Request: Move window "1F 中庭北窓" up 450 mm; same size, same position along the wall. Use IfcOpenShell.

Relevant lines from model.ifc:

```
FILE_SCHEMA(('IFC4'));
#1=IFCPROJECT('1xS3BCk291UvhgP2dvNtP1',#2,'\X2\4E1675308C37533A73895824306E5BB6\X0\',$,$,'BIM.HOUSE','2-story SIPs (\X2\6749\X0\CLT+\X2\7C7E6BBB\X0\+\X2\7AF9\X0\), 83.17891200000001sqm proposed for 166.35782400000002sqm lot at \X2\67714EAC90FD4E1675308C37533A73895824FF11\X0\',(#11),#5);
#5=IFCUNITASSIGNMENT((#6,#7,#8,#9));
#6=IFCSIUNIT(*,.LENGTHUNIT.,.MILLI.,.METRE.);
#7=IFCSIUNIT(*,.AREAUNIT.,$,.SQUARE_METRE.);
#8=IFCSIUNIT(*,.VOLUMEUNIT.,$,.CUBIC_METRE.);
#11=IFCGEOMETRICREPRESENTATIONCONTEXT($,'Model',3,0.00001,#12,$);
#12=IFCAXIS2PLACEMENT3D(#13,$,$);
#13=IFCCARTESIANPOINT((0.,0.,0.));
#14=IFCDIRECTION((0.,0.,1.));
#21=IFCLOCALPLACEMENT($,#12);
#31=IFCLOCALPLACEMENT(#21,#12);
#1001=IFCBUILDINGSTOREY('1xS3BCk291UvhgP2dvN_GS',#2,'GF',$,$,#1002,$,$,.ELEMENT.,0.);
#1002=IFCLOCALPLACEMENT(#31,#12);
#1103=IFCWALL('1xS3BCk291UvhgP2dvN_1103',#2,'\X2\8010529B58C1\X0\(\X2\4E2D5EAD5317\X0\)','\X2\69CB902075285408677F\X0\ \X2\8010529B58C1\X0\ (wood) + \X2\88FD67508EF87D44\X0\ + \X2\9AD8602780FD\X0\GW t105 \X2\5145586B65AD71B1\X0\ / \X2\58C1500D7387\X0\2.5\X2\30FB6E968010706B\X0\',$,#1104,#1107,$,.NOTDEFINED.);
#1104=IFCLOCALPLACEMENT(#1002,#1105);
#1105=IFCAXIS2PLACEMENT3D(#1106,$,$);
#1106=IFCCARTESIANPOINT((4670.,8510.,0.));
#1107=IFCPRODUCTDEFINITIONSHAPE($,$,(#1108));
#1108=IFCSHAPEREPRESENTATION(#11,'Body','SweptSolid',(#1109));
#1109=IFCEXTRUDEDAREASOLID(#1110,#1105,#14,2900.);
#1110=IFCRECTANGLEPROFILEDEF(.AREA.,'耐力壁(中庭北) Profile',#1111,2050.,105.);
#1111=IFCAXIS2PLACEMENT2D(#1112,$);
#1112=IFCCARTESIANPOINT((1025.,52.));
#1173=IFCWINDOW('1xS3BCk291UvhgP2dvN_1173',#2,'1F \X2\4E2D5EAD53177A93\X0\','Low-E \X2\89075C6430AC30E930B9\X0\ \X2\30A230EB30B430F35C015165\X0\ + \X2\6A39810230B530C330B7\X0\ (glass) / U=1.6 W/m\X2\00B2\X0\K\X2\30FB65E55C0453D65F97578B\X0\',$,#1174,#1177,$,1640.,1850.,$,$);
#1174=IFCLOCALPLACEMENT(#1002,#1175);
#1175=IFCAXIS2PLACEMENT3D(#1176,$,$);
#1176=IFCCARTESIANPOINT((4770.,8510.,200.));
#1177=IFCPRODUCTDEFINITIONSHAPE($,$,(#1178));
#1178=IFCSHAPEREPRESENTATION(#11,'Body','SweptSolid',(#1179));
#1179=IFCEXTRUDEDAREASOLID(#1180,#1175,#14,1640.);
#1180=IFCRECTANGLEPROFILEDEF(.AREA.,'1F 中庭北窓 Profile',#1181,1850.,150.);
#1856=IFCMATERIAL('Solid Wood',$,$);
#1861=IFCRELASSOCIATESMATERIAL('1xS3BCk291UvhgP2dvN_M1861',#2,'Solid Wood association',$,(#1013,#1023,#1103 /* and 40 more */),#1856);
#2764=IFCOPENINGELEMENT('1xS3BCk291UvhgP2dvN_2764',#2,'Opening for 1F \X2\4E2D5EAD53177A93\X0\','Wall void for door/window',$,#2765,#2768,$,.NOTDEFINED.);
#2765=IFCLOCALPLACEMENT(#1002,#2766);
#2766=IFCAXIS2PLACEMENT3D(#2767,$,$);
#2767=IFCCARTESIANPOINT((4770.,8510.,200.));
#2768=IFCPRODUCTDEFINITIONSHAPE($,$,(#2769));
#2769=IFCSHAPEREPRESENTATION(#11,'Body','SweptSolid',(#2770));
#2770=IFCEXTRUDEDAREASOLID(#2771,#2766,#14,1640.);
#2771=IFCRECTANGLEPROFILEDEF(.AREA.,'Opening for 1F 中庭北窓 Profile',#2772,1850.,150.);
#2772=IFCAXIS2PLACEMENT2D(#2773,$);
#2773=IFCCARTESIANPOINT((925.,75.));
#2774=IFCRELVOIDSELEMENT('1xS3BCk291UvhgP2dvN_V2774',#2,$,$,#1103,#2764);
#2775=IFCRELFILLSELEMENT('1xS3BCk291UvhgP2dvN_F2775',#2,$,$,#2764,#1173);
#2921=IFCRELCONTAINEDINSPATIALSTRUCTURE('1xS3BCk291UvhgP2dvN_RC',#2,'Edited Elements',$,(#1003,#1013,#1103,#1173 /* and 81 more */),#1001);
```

```python
import numpy as np
import ifcopenshell
import ifcopenshell.api.geometry
import ifcopenshell.util.placement
import ifcopenshell.util.unit

model = ifcopenshell.open("model.ifc")
unit_scale = ifcopenshell.util.unit.calculate_unit_scale(model)

window = model.by_id(1173)
opening = window.FillsVoids[0].RelatingOpeningElement
dz = 450.0

shift = np.array([0.0, 0.0, dz])
# The window is not placed relative to its opening, so move both.
for product in (opening, window):
    matrix = ifcopenshell.util.placement.get_local_placement(product.ObjectPlacement)
    matrix[:3, 3] += shift
    ifcopenshell.api.geometry.edit_object_placement(model, product=product, matrix=matrix, is_si=False)

print(f"moved by {dz * unit_scale:+.3f} m")

model.write("model-out.ifc")
```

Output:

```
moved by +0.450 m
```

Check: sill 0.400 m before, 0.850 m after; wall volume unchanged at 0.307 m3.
